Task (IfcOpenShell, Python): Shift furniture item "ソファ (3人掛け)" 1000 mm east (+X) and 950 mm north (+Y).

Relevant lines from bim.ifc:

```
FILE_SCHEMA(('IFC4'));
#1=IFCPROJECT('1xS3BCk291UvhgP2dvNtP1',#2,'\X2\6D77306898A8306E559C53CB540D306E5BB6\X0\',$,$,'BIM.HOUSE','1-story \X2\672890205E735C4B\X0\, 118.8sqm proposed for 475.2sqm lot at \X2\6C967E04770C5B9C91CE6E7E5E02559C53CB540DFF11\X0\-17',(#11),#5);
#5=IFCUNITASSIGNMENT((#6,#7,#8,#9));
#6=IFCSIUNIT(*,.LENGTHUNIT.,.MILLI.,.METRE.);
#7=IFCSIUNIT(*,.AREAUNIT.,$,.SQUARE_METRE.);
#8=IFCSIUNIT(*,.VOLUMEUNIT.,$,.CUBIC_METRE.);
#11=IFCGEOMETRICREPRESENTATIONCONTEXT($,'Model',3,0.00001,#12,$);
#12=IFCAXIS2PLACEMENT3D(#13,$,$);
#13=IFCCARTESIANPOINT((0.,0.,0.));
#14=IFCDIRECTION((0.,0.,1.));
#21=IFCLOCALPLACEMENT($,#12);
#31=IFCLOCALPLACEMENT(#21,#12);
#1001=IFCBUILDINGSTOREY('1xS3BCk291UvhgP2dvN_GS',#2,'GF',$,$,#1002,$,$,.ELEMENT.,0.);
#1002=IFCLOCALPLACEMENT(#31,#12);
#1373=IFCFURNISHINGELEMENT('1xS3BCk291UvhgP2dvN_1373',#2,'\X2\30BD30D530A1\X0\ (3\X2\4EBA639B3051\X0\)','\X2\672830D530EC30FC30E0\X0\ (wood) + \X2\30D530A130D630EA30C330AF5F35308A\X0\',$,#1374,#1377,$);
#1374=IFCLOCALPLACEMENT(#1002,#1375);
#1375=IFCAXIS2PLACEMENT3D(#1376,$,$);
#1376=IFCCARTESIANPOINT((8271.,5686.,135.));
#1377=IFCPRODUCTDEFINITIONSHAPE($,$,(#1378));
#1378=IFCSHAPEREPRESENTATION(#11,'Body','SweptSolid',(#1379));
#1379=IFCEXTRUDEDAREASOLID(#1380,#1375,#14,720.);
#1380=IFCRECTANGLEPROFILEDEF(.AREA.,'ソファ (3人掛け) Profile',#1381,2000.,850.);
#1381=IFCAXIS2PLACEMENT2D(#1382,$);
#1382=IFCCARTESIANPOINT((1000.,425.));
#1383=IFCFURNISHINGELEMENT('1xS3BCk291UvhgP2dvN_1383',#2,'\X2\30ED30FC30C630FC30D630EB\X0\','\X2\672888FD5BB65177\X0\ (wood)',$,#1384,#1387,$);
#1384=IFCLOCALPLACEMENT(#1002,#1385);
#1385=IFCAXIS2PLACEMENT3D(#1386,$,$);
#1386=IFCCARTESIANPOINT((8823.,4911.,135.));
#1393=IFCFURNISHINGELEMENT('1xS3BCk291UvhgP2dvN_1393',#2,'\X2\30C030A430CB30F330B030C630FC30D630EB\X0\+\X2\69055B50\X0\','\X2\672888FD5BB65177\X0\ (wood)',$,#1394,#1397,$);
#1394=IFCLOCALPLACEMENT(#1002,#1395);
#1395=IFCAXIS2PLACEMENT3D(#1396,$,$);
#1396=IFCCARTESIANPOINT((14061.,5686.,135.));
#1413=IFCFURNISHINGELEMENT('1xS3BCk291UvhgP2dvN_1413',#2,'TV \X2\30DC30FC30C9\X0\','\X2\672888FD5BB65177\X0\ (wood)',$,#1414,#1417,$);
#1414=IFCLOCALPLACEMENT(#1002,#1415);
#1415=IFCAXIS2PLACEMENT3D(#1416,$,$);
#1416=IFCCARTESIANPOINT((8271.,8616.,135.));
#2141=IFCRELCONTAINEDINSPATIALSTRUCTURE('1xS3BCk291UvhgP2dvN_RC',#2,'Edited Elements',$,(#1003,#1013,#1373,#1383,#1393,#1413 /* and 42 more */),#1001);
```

```python
import ifcopenshell
import ifcopenshell.api.geometry
import ifcopenshell.util.placement
import ifcopenshell.util.unit

model = ifcopenshell.open("bim.ifc")
unit_scale = ifcopenshell.util.unit.calculate_unit_scale(model)

item = model.by_id(1373)
matrix = ifcopenshell.util.placement.get_local_placement(item.ObjectPlacement)
matrix[0, 3] += 1 / unit_scale
matrix[1, 3] += 0.95 / unit_scale
ifcopenshell.api.geometry.edit_object_placement(model, product=item, matrix=matrix, is_si=False)

print(ifcopenshell.util.placement.get_local_placement(item.ObjectPlacement).round(3) + 0.0)

model.write("bim_edited.ifc")
```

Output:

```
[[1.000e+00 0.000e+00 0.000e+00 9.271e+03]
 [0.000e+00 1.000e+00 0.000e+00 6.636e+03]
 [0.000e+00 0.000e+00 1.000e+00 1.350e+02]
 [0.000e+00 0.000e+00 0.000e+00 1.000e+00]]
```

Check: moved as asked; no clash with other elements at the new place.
